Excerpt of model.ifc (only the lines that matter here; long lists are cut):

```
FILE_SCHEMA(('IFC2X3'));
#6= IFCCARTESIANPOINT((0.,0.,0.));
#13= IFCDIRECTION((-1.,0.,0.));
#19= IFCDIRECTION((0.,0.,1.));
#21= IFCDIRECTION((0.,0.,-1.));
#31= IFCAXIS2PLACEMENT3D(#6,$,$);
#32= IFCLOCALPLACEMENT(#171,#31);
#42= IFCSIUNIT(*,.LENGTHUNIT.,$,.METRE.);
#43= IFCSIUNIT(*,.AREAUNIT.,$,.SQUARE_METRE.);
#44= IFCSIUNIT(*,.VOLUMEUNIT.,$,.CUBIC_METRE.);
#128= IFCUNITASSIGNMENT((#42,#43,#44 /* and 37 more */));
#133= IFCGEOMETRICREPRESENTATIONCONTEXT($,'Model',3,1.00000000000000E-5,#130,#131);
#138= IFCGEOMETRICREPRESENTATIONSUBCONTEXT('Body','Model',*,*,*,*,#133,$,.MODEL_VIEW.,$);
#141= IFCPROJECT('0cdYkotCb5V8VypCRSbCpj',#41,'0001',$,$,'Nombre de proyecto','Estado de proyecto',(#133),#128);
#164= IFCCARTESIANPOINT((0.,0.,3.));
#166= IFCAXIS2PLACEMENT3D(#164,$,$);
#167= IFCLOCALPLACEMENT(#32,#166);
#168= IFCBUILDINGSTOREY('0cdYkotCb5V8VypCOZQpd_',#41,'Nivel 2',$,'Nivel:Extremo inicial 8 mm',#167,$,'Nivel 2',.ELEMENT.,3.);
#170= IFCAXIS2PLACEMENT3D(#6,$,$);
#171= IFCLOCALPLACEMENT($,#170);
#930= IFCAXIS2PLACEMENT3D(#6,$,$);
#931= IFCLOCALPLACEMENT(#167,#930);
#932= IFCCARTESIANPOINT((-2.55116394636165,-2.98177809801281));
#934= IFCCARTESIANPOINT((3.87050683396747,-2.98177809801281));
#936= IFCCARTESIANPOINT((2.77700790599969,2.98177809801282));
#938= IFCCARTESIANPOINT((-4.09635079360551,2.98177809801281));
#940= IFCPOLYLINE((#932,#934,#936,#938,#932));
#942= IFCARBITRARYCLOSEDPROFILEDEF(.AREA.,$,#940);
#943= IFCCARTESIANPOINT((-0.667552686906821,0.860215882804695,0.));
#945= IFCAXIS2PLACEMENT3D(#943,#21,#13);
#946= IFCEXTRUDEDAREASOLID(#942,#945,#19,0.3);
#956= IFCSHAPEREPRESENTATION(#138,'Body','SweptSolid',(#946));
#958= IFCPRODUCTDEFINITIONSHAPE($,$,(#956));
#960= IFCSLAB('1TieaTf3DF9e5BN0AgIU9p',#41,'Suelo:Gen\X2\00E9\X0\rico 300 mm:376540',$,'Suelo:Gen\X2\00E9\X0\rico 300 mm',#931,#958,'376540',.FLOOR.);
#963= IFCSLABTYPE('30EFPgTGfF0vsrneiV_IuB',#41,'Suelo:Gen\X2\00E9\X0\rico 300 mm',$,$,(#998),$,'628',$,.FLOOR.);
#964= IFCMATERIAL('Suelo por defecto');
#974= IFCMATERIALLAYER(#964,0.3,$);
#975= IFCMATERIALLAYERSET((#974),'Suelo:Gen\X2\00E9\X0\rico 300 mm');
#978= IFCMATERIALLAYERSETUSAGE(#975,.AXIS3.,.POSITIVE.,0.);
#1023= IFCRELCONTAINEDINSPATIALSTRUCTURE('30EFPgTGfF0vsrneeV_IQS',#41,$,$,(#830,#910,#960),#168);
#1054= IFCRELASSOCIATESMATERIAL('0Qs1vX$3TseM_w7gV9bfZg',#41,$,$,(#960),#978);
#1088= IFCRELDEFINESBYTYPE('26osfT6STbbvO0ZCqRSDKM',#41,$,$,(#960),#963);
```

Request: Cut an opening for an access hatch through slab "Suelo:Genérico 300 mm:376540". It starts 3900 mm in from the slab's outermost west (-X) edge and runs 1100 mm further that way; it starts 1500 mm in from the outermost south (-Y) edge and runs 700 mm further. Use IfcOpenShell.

```python
import numpy as np
import ifcopenshell
import ifcopenshell.api.feature
import ifcopenshell.api.geometry
import ifcopenshell.api.root
import ifcopenshell.geom
import ifcopenshell.util.placement
import ifcopenshell.util.representation
import ifcopenshell.util.shape
import ifcopenshell.util.unit

model = ifcopenshell.open("model.ifc")
unit_scale = ifcopenshell.util.unit.calculate_unit_scale(model)
settings = ifcopenshell.geom.settings()


def volume(element):
    """Net volume in cubic metres, openings subtracted."""
    shape = ifcopenshell.geom.create_shape(settings, element)
    return ifcopenshell.util.shape.get_volume(shape.geometry)


slab = model.by_guid("1TieaTf3DF9e5BN0AgIU9p")
before = volume(slab)

# Extent in the slab's own axes, in metres. The edges named are its -X and -Y sides.
slab_shape = ifcopenshell.geom.create_shape(settings, slab)
vertices = ifcopenshell.util.shape.get_vertices(slab_shape.geometry)
x_min, y_min, bottom = vertices.min(axis=0)
top = vertices[:, 2].max()

opening = ifcopenshell.api.root.create_entity(model, ifc_class="IfcOpeningElement", name="Access hatch opening")
context = ifcopenshell.util.representation.get_context(model, "Model", "Body", "MODEL_VIEW")
width, depth = 1.1, 0.7
outline = [(0.0, 0.0), (width, 0.0), (width, depth), (0.0, depth), (0.0, 0.0)]
# Overshoot both faces by 50 mm so the cut is clean.
shape = ifcopenshell.api.geometry.add_slab_representation(
    model, context=context, depth=top - bottom + 0.1, polyline=outline
)
ifcopenshell.api.geometry.assign_representation(model, product=opening, representation=shape)

matrix = ifcopenshell.util.placement.get_local_placement(slab.ObjectPlacement)
matrix[:, 3] = matrix @ np.append(np.array([x_min + 3.9, y_min + 1.5, bottom - 0.05]) / unit_scale, 1.0)
ifcopenshell.api.geometry.edit_object_placement(model, product=opening, matrix=matrix, is_si=False)
ifcopenshell.api.feature.add_feature(model, feature=opening, element=slab)

after = volume(slab)

print(f"slab volume {before:.3f} -> {after:.3f} m3")

model.write("model_rev.ifc")
```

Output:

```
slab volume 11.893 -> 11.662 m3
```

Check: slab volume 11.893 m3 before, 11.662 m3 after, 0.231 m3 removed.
